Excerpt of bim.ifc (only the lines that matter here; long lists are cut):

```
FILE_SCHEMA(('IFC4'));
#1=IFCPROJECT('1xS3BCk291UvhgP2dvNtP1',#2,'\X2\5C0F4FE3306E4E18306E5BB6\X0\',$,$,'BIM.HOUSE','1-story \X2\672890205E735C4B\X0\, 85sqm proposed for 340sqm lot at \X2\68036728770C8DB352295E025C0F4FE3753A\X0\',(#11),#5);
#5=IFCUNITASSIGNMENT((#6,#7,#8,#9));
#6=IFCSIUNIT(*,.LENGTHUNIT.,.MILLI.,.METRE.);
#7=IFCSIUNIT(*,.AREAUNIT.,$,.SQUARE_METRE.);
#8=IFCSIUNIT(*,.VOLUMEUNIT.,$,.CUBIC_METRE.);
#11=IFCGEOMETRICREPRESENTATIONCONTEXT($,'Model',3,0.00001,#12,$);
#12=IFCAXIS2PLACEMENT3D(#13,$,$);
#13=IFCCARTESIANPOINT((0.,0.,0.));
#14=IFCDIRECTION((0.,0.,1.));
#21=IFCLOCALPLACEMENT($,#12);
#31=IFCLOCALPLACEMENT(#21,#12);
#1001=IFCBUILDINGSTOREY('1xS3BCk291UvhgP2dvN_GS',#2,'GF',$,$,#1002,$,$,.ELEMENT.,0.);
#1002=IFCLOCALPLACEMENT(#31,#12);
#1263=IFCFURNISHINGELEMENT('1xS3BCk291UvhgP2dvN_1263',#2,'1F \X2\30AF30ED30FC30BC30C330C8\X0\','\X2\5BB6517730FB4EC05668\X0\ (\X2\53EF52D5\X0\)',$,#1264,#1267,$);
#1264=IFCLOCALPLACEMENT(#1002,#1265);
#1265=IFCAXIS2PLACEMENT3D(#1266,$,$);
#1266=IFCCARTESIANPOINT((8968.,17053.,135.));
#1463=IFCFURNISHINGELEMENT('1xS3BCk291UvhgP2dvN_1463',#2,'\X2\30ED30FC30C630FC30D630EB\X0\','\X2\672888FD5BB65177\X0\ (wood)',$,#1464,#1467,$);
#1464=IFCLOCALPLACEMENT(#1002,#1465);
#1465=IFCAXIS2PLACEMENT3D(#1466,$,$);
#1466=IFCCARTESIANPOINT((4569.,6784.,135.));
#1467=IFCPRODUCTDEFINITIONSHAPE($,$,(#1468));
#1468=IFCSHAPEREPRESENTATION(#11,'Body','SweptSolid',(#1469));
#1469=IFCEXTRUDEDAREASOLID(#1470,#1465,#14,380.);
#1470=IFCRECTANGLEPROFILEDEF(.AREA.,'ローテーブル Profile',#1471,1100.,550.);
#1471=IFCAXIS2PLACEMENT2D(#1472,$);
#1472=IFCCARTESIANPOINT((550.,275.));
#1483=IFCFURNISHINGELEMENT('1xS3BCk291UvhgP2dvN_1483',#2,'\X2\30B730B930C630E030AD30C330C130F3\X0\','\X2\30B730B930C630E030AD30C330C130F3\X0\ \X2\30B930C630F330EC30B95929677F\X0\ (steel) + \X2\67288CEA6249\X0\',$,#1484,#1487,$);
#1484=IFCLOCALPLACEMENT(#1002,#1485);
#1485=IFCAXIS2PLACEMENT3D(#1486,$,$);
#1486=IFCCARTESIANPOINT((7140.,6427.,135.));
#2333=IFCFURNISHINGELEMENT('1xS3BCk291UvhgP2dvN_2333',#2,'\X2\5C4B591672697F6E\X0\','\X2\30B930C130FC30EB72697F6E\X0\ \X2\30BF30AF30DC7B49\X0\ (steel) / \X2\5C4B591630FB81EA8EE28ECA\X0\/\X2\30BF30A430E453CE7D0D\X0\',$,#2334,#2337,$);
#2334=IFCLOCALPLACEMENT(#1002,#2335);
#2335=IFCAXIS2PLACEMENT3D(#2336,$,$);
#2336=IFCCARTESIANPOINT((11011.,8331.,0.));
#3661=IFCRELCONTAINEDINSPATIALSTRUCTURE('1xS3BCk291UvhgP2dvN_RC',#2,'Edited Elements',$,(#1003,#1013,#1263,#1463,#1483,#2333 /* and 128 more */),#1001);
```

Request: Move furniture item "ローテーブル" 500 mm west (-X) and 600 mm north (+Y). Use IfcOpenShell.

```python
import ifcopenshell
import ifcopenshell.api.geometry
import ifcopenshell.util.placement
import ifcopenshell.util.unit

model = ifcopenshell.open("bim.ifc")
unit_scale = ifcopenshell.util.unit.calculate_unit_scale(model)

item = model.by_guid("1xS3BCk291UvhgP2dvN_1463")
matrix = ifcopenshell.util.placement.get_local_placement(item.ObjectPlacement)
matrix[0, 3] -= 0.5 / unit_scale
matrix[1, 3] += 0.6 / unit_scale
ifcopenshell.api.geometry.edit_object_placement(model, product=item, matrix=matrix, is_si=False)

print(ifcopenshell.util.placement.get_local_placement(item.ObjectPlacement).round(3) + 0.0)

model.write("bim_edited.ifc")
```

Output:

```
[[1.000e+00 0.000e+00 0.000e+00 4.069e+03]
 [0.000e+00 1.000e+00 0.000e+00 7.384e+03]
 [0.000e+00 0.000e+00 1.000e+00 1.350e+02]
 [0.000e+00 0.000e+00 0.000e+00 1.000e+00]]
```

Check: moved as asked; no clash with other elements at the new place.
